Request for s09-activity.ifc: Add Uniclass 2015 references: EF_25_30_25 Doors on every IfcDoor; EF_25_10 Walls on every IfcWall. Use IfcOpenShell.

First a look at what the model holds.

```python
import ifcopenshell

model = ifcopenshell.open("s09-activity.ifc")
print(model.schema)
print("classifications:", [c.Name for c in model.by_type("IfcClassification")])
for ifc_class in ("IfcDoor", "IfcRoof", "IfcStair", "IfcWall", "IfcWindow"):
    print(ifc_class, len(model.by_type(ifc_class)))
```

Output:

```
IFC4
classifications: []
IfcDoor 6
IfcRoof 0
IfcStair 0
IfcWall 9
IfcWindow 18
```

```python
import ifcopenshell
import ifcopenshell.api.classification

model = ifcopenshell.open("s09-activity.ifc")

system = ifcopenshell.api.classification.add_classification(model, classification="Uniclass 2015")

codes = {
    "IfcDoor": ("EF_25_30_25", "Doors"),
    "IfcWall": ("EF_25_10", "Walls"),
}
for ifc_class, (code, name) in codes.items():
    products = model.by_type(ifc_class)
    ifcopenshell.api.classification.add_reference(
        model, products=products, classification=system, identification=code, name=name
    )
    print(code, len(products))

model.write("s09-activity_rev.ifc")
```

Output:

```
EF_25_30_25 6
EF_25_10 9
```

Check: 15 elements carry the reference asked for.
